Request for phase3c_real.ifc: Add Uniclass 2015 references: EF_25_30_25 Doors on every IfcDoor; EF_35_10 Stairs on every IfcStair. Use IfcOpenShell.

First a look at what the model holds.

```python
import ifcopenshell

model = ifcopenshell.open("phase3c_real.ifc")
print(model.schema)
print("classifications:", [c.Name for c in model.by_type("IfcClassification")])
for ifc_class in ("IfcDoor", "IfcRoof", "IfcStair", "IfcWall", "IfcWindow"):
    print(ifc_class, len(model.by_type(ifc_class)))
```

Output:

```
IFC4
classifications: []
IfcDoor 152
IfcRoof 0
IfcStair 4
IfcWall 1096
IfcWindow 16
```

```python
import ifcopenshell
import ifcopenshell.api.classification

model = ifcopenshell.open("phase3c_real.ifc")

system = ifcopenshell.api.classification.add_classification(model, classification="Uniclass 2015")

codes = {
    "IfcDoor": ("EF_25_30_25", "Doors"),
    "IfcStair": ("EF_35_10", "Stairs"),
}
for ifc_class, (code, name) in codes.items():
    products = model.by_type(ifc_class)
    ifcopenshell.api.classification.add_reference(
        model, products=products, classification=system, identification=code, name=name
    )
    print(code, len(products))

model.write("phase3c_real_updated.ifc")
```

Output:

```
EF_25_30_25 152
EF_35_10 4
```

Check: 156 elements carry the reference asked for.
